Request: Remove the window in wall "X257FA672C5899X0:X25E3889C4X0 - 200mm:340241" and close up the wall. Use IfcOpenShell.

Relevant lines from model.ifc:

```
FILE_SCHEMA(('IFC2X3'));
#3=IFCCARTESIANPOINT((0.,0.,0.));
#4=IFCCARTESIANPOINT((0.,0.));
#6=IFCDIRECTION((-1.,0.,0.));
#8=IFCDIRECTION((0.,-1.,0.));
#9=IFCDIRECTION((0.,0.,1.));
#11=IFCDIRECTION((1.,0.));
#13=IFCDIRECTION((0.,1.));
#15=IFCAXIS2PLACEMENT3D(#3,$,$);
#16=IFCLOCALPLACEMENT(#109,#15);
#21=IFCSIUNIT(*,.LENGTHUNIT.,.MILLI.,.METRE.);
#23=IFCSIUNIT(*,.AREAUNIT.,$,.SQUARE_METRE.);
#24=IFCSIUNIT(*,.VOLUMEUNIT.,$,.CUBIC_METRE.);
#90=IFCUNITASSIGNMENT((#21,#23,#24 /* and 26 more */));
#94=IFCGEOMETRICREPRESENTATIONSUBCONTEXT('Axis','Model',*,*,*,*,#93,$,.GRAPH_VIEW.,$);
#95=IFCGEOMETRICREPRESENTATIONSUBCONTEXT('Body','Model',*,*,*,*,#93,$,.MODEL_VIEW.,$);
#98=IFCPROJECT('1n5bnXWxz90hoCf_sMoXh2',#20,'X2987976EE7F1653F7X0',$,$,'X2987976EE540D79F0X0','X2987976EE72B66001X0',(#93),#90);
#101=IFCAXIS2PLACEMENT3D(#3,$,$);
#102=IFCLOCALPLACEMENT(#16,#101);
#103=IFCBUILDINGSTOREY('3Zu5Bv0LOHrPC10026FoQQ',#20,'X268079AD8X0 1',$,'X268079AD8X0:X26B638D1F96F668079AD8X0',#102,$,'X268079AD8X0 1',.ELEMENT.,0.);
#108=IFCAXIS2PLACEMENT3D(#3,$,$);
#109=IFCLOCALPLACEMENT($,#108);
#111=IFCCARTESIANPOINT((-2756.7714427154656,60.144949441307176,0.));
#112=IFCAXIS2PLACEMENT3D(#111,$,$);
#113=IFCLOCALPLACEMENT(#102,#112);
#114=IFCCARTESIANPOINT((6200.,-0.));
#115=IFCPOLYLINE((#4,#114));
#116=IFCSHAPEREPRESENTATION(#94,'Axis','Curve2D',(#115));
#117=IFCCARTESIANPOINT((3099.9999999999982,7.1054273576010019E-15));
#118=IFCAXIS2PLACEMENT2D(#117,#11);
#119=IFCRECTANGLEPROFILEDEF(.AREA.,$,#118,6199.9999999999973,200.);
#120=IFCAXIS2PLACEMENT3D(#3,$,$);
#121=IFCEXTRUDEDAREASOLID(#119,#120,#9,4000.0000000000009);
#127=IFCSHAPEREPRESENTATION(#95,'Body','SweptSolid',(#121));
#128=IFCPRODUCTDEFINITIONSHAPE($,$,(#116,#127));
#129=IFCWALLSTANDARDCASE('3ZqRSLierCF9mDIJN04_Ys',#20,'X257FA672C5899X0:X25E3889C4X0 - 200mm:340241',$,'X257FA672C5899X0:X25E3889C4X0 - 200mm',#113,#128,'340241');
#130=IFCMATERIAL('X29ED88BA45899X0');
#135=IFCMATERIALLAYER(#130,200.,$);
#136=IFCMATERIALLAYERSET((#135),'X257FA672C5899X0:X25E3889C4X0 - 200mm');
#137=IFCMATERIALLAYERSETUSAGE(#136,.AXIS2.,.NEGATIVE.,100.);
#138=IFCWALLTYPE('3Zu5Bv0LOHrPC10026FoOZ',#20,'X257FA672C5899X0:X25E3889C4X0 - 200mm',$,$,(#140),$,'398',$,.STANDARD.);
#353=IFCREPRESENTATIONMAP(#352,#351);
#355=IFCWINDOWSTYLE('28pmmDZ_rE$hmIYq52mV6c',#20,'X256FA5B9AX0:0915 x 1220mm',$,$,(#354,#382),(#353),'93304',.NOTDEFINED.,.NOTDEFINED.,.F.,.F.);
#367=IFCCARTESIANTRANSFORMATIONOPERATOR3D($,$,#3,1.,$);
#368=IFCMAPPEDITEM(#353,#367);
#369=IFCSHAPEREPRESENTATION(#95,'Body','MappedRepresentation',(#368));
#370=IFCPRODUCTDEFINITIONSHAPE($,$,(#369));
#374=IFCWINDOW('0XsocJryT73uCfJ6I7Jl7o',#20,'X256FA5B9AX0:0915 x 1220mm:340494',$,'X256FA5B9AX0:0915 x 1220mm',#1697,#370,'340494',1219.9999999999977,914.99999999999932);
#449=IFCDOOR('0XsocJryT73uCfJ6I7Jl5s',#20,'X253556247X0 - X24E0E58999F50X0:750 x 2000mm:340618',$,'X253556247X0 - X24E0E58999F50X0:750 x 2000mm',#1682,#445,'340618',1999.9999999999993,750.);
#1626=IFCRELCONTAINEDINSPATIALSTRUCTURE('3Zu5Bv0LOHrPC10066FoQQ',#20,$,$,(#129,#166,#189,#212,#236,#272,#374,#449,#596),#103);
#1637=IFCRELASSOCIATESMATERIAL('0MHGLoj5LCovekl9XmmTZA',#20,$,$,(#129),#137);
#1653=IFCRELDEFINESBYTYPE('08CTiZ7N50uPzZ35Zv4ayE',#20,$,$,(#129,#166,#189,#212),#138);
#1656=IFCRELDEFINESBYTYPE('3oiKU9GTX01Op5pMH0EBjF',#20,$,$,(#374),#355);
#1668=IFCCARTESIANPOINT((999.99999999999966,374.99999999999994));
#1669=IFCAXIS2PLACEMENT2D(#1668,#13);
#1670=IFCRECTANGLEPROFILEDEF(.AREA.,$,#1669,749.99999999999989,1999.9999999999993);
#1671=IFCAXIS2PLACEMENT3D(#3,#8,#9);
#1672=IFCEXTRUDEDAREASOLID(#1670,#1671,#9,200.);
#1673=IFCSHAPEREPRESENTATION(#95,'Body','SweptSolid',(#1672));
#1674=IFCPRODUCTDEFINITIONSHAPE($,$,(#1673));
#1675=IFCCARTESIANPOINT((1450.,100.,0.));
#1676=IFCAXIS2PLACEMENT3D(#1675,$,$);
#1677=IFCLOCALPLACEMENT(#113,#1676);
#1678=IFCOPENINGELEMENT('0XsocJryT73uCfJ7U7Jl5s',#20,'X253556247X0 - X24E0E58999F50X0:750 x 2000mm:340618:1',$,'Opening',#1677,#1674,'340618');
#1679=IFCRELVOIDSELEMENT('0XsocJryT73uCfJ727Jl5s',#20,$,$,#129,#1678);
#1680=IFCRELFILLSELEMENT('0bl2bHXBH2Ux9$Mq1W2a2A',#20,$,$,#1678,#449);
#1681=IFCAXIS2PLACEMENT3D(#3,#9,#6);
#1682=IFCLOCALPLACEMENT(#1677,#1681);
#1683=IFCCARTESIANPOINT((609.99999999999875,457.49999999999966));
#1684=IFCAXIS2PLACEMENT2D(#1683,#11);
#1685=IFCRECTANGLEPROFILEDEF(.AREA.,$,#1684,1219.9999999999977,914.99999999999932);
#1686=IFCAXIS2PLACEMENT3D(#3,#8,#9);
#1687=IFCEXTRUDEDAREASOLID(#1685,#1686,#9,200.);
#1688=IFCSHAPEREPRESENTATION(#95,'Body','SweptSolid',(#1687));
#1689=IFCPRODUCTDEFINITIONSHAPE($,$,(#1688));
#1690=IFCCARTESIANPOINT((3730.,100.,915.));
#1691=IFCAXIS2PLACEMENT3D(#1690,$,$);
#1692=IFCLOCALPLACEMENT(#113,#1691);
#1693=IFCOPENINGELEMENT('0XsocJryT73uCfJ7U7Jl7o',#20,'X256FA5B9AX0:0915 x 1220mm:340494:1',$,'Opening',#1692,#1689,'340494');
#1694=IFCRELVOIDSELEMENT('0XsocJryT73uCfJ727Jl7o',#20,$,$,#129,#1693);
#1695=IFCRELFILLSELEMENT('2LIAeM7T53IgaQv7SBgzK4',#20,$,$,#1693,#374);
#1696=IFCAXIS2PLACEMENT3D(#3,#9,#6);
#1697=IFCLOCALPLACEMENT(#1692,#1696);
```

```python
import ifcopenshell
import ifcopenshell.api.feature
import ifcopenshell.api.root
import ifcopenshell.geom
import ifcopenshell.util.shape

model = ifcopenshell.open("model.ifc")
settings = ifcopenshell.geom.settings()


def volume(element):
    """Net volume in cubic metres, openings subtracted."""
    shape = ifcopenshell.geom.create_shape(settings, element)
    return ifcopenshell.util.shape.get_volume(shape.geometry)


window = model.by_id(374)
opening = window.FillsVoids[0].RelatingOpeningElement
wall = opening.VoidsElements[0].RelatingBuildingElement
before = volume(wall)

ifcopenshell.api.root.remove_product(model, product=window)
ifcopenshell.api.feature.remove_feature(model, feature=opening)

after = volume(wall)

print(f"wall volume {before:.3f} -> {after:.3f} m3")

model.write("model-out.ifc")
```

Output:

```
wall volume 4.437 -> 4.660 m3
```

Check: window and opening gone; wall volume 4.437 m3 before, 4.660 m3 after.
